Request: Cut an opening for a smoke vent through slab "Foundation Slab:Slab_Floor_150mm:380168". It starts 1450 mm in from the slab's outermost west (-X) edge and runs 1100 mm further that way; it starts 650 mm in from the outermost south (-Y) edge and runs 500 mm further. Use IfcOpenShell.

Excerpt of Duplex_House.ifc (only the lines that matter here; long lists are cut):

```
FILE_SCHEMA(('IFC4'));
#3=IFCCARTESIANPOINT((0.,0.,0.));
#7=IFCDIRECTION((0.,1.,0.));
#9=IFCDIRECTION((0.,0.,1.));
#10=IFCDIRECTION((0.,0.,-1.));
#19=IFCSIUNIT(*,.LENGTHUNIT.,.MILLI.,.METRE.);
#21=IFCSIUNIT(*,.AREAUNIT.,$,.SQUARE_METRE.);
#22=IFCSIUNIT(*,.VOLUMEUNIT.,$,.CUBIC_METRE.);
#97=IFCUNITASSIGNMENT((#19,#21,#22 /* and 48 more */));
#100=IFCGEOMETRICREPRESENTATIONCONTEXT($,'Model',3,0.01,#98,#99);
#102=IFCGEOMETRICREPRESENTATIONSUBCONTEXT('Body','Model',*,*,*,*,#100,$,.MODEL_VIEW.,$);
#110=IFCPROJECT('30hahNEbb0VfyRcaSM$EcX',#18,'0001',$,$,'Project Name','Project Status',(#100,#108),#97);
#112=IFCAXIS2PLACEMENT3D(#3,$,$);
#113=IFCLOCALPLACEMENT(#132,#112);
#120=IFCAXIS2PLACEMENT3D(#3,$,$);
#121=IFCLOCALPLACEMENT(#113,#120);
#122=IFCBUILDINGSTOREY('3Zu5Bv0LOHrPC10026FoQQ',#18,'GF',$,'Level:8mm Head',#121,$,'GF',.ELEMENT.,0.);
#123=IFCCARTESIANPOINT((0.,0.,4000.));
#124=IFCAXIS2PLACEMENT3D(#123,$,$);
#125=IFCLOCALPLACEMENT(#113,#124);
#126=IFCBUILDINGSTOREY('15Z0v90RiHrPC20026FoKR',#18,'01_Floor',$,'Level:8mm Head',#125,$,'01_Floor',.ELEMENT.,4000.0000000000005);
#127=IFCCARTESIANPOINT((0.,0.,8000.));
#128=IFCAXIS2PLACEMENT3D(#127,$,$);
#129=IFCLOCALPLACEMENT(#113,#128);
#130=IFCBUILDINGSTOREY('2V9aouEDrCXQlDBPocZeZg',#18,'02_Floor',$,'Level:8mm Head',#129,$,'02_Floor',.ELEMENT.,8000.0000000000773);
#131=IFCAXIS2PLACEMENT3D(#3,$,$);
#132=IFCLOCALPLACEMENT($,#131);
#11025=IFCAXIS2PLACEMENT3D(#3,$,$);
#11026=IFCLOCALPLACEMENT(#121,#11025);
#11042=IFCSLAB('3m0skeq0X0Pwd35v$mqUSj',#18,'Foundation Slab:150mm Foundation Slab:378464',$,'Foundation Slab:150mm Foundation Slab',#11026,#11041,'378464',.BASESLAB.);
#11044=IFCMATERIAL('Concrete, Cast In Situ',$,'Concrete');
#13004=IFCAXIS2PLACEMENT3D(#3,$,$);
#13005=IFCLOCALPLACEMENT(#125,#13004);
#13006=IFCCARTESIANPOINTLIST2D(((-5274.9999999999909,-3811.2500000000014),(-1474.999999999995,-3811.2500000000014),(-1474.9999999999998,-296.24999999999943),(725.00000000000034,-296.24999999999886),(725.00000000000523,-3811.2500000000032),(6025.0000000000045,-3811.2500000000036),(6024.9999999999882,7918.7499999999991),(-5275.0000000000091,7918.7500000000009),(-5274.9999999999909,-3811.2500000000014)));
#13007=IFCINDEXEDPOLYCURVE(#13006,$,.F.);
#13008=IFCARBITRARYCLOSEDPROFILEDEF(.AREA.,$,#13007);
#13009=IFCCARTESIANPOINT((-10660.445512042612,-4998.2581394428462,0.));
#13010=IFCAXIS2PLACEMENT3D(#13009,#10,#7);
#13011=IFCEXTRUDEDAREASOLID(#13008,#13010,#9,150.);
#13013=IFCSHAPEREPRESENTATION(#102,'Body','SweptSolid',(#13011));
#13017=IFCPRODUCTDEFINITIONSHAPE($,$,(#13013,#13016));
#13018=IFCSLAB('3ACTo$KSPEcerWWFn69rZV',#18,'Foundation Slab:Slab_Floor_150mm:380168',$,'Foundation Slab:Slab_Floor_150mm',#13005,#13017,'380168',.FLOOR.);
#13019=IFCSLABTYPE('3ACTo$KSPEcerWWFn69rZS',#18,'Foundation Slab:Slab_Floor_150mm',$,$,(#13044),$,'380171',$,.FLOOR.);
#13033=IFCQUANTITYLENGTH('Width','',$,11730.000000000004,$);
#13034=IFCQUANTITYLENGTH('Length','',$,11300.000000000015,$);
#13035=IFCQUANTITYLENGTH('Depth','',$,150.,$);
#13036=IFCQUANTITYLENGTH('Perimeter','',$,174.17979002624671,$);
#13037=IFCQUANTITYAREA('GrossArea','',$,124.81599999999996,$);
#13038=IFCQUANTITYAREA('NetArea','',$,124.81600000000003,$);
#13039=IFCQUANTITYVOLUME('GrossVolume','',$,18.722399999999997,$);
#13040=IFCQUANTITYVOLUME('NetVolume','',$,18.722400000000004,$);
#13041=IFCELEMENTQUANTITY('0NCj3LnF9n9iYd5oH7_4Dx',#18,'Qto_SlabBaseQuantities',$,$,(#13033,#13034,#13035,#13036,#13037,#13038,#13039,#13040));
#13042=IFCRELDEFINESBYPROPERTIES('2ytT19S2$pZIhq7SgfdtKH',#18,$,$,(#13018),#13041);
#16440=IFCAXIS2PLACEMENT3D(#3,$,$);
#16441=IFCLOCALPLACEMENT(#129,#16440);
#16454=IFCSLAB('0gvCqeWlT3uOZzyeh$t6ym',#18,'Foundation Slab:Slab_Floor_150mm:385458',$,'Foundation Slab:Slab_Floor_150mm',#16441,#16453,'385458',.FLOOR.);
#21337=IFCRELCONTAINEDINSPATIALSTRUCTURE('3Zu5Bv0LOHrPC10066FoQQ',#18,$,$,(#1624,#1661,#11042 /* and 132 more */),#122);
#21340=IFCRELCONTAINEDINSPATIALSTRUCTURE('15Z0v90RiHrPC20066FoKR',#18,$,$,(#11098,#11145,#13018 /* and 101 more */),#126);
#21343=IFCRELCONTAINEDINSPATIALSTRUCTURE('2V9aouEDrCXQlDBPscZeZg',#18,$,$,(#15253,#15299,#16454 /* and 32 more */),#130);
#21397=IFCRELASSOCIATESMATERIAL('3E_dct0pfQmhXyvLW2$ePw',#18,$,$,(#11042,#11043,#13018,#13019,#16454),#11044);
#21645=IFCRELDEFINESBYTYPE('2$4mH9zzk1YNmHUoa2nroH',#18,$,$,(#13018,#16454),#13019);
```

```python
import numpy as np
import ifcopenshell
import ifcopenshell.api.feature
import ifcopenshell.api.geometry
import ifcopenshell.api.pset
import ifcopenshell.api.root
import ifcopenshell.geom
import ifcopenshell.util.element
import ifcopenshell.util.placement
import ifcopenshell.util.representation
import ifcopenshell.util.shape
import ifcopenshell.util.unit

model = ifcopenshell.open("Duplex_House.ifc")
unit_scale = ifcopenshell.util.unit.calculate_unit_scale(model)
area_scale = ifcopenshell.util.unit.calculate_unit_scale(model, "AREAUNIT")
volume_scale = ifcopenshell.util.unit.calculate_unit_scale(model, "VOLUMEUNIT")
settings = ifcopenshell.geom.settings()


def volume(element):
    """Net volume in cubic metres, openings subtracted."""
    shape = ifcopenshell.geom.create_shape(settings, element)
    return ifcopenshell.util.shape.get_volume(shape.geometry)


slab = model.by_guid("3ACTo$KSPEcerWWFn69rZV")
before = volume(slab)

# Extent in the slab's own axes, in metres. The edges named are its -X and -Y sides.
slab_shape = ifcopenshell.geom.create_shape(settings, slab)
vertices = ifcopenshell.util.shape.get_vertices(slab_shape.geometry)
x_min, y_min, bottom = vertices.min(axis=0)
top = vertices[:, 2].max()

opening = ifcopenshell.api.root.create_entity(model, ifc_class="IfcOpeningElement", name="Smoke vent opening", predefined_type="OPENING")
context = ifcopenshell.util.representation.get_context(model, "Model", "Body", "MODEL_VIEW")
width, depth = 1.1, 0.5
outline = [(0.0, 0.0), (width, 0.0), (width, depth), (0.0, depth), (0.0, 0.0)]
# Overshoot both faces by 50 mm so the cut is clean.
shape = ifcopenshell.api.geometry.add_slab_representation(
    model, context=context, depth=top - bottom + 0.1, polyline=outline
)
ifcopenshell.api.geometry.assign_representation(model, product=opening, representation=shape)

matrix = ifcopenshell.util.placement.get_local_placement(slab.ObjectPlacement)
matrix[:, 3] = matrix @ np.append(np.array([x_min + 1.45, y_min + 0.65, bottom - 0.05]) / unit_scale, 1.0)
ifcopenshell.api.geometry.edit_object_placement(model, product=opening, matrix=matrix, is_si=False)
ifcopenshell.api.feature.add_feature(model, feature=opening, element=slab)

after = volume(slab)

# Update the slab's stored quantities.
qto = model.by_id(ifcopenshell.util.element.get_pset(slab, "Qto_SlabBaseQuantities", should_inherit=False)["id"])
ifcopenshell.api.pset.edit_qto(model, qto=qto, properties={
    "NetArea": after / (top - bottom) / area_scale,
    "NetVolume": after / volume_scale,
})

print(f"slab volume {before:.3f} -> {after:.3f} m3")

model.write("Duplex_House_v2.ifc")
```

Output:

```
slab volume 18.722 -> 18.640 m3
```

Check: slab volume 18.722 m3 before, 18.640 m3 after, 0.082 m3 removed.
